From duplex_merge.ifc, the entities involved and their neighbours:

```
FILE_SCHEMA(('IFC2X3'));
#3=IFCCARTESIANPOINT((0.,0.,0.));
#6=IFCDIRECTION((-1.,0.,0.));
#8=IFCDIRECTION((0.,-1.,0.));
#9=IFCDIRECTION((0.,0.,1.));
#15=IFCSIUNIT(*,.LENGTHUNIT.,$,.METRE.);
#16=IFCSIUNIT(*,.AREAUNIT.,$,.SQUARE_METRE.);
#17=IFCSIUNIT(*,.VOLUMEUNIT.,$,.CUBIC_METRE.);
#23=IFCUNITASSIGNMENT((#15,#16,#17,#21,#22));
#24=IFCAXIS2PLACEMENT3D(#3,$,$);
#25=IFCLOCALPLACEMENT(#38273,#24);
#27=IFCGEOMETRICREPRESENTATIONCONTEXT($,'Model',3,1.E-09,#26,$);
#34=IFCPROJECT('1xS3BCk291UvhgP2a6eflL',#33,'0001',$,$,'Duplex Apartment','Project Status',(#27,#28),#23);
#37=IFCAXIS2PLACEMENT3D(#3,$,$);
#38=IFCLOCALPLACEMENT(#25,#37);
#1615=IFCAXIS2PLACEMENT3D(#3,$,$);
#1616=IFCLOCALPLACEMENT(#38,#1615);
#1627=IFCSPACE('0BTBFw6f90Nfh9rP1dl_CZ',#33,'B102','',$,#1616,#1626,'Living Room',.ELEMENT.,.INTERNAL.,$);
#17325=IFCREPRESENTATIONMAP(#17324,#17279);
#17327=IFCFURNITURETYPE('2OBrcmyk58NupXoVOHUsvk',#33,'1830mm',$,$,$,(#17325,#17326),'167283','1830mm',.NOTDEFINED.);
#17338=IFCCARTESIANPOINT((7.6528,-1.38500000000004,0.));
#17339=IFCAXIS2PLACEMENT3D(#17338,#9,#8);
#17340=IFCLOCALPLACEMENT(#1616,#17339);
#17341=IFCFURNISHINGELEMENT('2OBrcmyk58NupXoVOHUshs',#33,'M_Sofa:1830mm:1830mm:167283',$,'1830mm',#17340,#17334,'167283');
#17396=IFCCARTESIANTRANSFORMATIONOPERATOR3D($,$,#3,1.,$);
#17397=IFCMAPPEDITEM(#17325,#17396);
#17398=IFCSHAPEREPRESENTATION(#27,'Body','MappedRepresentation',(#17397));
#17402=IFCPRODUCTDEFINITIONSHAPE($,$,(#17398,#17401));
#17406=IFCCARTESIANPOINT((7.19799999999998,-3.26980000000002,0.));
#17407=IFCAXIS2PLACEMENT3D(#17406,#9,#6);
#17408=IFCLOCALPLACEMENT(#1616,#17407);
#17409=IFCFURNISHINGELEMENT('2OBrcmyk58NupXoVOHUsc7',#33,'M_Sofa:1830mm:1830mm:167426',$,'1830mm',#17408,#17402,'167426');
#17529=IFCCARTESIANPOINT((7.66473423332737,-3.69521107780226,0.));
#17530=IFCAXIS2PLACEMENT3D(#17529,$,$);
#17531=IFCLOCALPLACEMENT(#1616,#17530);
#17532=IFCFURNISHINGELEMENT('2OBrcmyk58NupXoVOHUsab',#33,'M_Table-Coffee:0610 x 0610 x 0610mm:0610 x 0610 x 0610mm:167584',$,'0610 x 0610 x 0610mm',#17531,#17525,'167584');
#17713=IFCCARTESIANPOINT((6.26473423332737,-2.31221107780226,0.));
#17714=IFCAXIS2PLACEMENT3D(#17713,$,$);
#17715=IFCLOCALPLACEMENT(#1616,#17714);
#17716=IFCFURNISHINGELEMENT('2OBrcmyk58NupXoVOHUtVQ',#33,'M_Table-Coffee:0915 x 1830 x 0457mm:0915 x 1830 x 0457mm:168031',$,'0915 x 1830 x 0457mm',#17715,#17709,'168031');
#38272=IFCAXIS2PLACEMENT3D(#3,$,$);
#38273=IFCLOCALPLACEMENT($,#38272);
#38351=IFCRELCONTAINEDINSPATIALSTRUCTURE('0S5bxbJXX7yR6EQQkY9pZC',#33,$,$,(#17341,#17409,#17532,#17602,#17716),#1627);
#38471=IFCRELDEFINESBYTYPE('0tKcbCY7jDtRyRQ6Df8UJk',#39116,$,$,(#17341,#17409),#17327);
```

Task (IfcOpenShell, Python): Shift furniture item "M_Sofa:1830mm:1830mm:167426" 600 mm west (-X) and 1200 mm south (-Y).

```python
import ifcopenshell
import ifcopenshell.api.geometry
import ifcopenshell.util.placement

model = ifcopenshell.open("duplex_merge.ifc")

item = model.by_guid("2OBrcmyk58NupXoVOHUsc7")
matrix = ifcopenshell.util.placement.get_local_placement(item.ObjectPlacement)
matrix[0, 3] -= 0.6
matrix[1, 3] -= 1.2
ifcopenshell.api.geometry.edit_object_placement(model, product=item, matrix=matrix, is_si=False)

print(ifcopenshell.util.placement.get_local_placement(item.ObjectPlacement).round(3) + 0.0)

model.write("duplex_merge_v2.ifc")
```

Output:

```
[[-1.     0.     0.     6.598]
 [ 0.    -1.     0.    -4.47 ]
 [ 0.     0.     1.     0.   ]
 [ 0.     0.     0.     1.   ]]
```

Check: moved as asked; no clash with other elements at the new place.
